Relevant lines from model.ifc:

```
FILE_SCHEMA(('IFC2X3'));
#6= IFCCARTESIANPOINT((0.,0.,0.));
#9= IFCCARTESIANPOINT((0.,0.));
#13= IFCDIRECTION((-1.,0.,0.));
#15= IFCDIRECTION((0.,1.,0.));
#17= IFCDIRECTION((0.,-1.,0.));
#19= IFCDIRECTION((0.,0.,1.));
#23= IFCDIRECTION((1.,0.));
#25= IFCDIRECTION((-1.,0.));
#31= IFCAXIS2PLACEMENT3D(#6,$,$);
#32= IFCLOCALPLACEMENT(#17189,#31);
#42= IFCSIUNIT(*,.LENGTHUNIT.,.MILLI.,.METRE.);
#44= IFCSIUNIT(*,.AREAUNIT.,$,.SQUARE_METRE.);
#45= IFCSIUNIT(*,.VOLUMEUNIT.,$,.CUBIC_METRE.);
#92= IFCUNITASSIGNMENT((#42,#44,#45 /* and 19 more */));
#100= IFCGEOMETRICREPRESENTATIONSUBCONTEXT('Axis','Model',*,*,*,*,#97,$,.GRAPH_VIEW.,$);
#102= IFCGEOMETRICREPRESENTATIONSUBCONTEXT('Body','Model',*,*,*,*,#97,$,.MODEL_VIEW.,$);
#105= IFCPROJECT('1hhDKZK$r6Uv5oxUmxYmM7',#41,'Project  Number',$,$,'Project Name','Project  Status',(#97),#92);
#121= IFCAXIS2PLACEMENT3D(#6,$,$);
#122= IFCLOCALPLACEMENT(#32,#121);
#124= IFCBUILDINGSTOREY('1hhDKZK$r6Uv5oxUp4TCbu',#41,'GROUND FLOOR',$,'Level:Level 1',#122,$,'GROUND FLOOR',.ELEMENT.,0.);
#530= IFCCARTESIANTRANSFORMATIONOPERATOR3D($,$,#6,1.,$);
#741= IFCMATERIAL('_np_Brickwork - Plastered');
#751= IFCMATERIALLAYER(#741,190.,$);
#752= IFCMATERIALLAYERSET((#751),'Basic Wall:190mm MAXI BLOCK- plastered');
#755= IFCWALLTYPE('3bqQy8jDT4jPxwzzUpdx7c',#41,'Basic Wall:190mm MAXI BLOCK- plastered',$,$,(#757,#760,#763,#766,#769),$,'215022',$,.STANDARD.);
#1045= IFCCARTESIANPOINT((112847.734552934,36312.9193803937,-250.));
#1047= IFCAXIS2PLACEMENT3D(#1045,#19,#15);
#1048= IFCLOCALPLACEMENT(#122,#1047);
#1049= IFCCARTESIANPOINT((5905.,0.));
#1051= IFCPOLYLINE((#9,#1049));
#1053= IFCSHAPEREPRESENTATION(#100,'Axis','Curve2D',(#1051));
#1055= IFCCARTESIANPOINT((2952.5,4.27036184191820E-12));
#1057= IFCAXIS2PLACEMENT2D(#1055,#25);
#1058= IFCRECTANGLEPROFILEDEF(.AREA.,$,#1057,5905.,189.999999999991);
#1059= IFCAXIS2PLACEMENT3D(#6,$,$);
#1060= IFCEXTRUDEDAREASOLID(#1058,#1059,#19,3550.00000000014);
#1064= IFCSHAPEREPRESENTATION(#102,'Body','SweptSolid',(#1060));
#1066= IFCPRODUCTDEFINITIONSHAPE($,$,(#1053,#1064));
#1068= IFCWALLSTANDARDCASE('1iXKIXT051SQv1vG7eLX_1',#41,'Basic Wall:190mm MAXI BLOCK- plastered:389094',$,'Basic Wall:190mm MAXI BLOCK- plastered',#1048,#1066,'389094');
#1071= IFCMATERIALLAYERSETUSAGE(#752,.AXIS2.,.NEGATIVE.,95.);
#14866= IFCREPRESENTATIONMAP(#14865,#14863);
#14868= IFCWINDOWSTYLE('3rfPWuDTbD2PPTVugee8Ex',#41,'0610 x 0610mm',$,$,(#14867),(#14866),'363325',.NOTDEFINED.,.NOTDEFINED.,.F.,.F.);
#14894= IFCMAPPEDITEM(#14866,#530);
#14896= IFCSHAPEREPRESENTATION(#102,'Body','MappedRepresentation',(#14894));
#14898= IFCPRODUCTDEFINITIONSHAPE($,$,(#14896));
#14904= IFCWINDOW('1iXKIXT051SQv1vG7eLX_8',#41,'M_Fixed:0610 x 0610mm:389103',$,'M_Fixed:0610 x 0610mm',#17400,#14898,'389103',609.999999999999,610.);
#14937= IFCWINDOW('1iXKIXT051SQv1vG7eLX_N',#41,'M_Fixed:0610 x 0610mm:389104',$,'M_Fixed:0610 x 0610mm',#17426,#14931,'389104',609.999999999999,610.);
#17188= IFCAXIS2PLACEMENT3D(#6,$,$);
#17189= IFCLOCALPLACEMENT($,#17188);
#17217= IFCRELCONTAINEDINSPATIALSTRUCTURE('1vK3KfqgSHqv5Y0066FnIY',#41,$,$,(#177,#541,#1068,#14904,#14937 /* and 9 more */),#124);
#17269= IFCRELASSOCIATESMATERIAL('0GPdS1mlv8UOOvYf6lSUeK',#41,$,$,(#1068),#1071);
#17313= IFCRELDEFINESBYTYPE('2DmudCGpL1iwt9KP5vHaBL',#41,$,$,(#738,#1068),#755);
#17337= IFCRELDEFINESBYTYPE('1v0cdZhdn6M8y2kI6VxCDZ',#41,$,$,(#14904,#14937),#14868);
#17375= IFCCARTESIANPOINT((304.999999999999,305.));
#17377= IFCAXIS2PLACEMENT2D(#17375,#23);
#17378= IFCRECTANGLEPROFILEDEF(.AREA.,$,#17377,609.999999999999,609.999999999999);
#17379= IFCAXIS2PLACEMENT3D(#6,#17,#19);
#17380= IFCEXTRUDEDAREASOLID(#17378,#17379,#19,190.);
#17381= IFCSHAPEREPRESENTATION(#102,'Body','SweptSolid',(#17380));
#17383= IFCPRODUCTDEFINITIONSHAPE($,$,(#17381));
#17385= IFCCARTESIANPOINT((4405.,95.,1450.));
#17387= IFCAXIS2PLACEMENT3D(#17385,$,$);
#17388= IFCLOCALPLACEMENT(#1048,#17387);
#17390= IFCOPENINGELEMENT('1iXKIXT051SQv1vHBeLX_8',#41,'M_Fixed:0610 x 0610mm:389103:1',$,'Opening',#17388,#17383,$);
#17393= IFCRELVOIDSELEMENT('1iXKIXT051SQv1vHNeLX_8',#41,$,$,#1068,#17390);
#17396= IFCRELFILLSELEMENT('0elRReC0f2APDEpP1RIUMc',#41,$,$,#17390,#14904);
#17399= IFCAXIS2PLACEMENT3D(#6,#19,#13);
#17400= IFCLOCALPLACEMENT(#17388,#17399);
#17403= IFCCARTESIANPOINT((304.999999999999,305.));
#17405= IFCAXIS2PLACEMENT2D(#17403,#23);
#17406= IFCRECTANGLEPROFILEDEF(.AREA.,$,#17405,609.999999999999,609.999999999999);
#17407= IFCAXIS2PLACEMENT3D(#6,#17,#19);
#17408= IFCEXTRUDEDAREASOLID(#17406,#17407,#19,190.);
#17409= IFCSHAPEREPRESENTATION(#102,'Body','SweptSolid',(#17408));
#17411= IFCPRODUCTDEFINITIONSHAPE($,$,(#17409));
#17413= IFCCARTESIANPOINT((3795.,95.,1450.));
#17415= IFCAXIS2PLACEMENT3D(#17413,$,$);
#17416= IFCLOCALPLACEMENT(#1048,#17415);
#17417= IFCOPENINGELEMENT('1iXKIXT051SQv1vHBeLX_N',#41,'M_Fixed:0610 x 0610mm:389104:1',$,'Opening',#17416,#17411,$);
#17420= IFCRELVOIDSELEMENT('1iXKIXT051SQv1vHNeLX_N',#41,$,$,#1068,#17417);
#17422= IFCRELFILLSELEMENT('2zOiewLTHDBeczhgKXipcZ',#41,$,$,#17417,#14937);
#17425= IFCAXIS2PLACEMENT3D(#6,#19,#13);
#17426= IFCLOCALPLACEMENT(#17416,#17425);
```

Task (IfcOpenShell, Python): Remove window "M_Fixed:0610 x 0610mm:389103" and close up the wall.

```python
import ifcopenshell
import ifcopenshell.api.feature
import ifcopenshell.api.root
import ifcopenshell.geom
import ifcopenshell.util.shape

model = ifcopenshell.open("model.ifc")
settings = ifcopenshell.geom.settings()


def volume(element):
    """Net volume in cubic metres, openings subtracted."""
    shape = ifcopenshell.geom.create_shape(settings, element)
    return ifcopenshell.util.shape.get_volume(shape.geometry)


window = model.by_guid("1iXKIXT051SQv1vG7eLX_8")
opening = window.FillsVoids[0].RelatingOpeningElement
wall = opening.VoidsElements[0].RelatingBuildingElement
before = volume(wall)

ifcopenshell.api.root.remove_product(model, product=window)
ifcopenshell.api.feature.remove_feature(model, feature=opening)

after = volume(wall)

print(f"wall volume {before:.3f} -> {after:.3f} m3")

model.write("model_rev.ifc")
```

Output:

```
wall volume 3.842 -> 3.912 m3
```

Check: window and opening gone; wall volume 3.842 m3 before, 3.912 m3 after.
